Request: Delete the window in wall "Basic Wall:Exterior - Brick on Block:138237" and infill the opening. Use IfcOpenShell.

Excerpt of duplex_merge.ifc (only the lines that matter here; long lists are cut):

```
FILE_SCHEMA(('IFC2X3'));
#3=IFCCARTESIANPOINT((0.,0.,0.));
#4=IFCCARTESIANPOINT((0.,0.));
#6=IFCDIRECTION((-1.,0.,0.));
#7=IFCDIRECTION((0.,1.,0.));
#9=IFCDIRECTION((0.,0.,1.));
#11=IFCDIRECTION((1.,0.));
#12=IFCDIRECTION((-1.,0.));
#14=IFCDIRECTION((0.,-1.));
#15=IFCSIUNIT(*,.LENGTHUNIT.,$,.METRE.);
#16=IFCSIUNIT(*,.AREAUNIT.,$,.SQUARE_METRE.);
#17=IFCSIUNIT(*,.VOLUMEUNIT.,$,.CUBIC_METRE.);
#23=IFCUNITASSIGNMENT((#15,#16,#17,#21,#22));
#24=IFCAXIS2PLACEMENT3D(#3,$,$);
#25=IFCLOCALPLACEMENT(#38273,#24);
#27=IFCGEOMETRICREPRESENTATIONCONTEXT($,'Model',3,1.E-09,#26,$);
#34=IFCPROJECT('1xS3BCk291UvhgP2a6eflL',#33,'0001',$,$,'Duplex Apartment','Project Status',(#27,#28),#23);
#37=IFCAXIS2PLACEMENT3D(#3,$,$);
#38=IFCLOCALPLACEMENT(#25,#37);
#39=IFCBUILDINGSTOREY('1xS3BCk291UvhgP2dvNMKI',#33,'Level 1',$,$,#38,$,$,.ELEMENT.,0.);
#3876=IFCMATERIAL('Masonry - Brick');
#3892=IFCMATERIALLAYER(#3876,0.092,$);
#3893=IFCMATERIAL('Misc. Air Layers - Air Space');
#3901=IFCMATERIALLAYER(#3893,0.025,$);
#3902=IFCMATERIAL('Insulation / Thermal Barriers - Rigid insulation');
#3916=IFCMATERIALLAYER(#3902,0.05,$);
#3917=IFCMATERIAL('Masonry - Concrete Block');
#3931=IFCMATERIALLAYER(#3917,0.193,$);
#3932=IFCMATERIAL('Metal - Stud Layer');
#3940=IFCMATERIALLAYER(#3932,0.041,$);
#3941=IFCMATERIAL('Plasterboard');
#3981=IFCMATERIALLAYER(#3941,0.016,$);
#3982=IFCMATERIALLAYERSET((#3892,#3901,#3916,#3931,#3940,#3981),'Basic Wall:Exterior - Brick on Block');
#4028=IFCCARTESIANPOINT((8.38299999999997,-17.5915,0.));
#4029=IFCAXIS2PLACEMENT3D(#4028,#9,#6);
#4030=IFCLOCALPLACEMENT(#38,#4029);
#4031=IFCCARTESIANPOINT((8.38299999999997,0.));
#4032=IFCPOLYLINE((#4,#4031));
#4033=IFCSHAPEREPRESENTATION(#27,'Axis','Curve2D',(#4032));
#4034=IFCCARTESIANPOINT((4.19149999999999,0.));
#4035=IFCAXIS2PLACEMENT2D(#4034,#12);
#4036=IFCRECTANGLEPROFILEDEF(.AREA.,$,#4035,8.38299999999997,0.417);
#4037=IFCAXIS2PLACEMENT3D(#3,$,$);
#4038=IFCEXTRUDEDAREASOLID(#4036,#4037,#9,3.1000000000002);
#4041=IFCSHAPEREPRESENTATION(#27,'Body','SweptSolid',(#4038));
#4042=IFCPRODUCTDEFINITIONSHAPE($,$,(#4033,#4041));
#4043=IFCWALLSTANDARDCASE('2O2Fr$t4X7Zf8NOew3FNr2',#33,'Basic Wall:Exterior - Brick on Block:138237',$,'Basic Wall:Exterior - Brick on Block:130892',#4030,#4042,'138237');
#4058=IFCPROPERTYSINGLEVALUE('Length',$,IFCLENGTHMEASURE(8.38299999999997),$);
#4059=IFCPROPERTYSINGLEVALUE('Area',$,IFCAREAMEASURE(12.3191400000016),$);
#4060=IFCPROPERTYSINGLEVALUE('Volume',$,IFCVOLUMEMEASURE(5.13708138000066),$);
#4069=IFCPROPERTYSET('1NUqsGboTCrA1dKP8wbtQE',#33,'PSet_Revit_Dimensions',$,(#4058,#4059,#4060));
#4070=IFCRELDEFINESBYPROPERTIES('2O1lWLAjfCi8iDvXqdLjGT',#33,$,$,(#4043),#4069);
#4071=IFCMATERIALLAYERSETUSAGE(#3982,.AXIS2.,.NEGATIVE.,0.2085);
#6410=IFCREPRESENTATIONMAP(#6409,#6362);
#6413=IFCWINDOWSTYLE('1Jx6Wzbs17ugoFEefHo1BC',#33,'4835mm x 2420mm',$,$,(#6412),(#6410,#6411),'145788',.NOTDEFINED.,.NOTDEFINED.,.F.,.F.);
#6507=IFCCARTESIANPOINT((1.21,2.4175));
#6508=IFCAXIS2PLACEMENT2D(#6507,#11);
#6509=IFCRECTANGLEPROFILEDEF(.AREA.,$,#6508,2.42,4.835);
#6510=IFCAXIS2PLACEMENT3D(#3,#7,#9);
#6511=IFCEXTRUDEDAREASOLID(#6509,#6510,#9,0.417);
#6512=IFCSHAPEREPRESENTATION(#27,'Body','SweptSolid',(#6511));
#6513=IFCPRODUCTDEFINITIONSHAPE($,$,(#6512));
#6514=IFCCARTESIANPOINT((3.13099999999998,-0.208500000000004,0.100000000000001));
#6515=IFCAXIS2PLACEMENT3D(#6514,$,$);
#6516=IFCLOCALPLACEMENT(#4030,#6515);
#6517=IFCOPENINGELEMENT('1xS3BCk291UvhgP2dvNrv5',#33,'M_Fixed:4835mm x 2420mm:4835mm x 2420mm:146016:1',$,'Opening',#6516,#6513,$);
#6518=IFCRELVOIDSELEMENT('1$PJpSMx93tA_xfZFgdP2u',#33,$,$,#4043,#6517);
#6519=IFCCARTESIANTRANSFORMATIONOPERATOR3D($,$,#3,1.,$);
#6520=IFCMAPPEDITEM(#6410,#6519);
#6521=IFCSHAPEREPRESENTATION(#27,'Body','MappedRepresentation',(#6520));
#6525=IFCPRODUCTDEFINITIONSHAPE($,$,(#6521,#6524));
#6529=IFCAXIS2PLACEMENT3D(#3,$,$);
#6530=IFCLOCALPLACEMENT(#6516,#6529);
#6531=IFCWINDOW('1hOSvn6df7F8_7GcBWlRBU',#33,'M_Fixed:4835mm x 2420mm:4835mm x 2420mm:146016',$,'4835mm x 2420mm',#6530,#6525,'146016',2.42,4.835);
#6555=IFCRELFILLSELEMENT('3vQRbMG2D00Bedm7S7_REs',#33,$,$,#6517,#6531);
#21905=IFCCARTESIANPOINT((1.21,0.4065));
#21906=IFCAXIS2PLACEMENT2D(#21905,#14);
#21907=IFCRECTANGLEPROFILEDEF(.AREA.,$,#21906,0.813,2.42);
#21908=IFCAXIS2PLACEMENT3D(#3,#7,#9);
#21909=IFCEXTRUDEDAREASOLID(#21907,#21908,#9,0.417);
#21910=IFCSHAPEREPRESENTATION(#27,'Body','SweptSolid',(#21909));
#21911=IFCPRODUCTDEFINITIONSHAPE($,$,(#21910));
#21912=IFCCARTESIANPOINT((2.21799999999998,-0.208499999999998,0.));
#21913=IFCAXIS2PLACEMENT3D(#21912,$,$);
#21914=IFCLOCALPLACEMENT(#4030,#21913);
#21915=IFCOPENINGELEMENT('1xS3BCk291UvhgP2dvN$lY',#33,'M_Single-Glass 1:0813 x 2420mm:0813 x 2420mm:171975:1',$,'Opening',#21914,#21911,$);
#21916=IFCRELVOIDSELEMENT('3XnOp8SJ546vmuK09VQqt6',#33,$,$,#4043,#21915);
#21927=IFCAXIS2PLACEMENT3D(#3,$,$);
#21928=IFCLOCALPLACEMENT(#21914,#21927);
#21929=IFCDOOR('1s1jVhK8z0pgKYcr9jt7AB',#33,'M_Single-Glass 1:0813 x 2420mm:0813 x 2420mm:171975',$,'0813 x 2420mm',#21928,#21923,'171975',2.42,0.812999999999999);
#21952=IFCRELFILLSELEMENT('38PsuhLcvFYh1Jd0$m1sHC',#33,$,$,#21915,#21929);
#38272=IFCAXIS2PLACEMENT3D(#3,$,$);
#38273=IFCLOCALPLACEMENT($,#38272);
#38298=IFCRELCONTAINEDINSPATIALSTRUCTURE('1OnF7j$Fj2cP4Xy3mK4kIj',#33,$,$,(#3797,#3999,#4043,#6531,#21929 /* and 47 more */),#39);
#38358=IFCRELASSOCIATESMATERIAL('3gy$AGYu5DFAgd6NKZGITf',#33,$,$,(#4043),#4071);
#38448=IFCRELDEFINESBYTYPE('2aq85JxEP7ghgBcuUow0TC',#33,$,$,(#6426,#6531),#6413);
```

```python
import ifcopenshell
import ifcopenshell.api.feature
import ifcopenshell.api.pset
import ifcopenshell.api.root
import ifcopenshell.geom
import ifcopenshell.util.element
import ifcopenshell.util.shape
import ifcopenshell.util.unit

model = ifcopenshell.open("duplex_merge.ifc")
area_scale = ifcopenshell.util.unit.calculate_unit_scale(model, "AREAUNIT")
volume_scale = ifcopenshell.util.unit.calculate_unit_scale(model, "VOLUMEUNIT")
settings = ifcopenshell.geom.settings()


def volume(element):
    """Net volume in cubic metres, openings subtracted."""
    shape = ifcopenshell.geom.create_shape(settings, element)
    return ifcopenshell.util.shape.get_volume(shape.geometry)


window = model.by_guid("1hOSvn6df7F8_7GcBWlRBU")
opening = window.FillsVoids[0].RelatingOpeningElement
wall = opening.VoidsElements[0].RelatingBuildingElement
before = volume(wall)

ifcopenshell.api.root.remove_product(model, product=window)
ifcopenshell.api.feature.remove_feature(model, feature=opening)

after = volume(wall)
thickness = 0.417  # wall thickness in metres

# Update the wall's stored quantities.
pset = model.by_id(ifcopenshell.util.element.get_pset(wall, "PSet_Revit_Dimensions", should_inherit=False)["id"])
ifcopenshell.api.pset.edit_pset(model, pset=pset, properties={
    "Area": model.create_entity("IfcAreaMeasure", after / thickness / area_scale),
    "Volume": model.create_entity("IfcVolumeMeasure", after / volume_scale),
})

print(f"wall volume {before:.3f} -> {after:.3f} m3")

model.write("duplex_merge_edited.ifc")
```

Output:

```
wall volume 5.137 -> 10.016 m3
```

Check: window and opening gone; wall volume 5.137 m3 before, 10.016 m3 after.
